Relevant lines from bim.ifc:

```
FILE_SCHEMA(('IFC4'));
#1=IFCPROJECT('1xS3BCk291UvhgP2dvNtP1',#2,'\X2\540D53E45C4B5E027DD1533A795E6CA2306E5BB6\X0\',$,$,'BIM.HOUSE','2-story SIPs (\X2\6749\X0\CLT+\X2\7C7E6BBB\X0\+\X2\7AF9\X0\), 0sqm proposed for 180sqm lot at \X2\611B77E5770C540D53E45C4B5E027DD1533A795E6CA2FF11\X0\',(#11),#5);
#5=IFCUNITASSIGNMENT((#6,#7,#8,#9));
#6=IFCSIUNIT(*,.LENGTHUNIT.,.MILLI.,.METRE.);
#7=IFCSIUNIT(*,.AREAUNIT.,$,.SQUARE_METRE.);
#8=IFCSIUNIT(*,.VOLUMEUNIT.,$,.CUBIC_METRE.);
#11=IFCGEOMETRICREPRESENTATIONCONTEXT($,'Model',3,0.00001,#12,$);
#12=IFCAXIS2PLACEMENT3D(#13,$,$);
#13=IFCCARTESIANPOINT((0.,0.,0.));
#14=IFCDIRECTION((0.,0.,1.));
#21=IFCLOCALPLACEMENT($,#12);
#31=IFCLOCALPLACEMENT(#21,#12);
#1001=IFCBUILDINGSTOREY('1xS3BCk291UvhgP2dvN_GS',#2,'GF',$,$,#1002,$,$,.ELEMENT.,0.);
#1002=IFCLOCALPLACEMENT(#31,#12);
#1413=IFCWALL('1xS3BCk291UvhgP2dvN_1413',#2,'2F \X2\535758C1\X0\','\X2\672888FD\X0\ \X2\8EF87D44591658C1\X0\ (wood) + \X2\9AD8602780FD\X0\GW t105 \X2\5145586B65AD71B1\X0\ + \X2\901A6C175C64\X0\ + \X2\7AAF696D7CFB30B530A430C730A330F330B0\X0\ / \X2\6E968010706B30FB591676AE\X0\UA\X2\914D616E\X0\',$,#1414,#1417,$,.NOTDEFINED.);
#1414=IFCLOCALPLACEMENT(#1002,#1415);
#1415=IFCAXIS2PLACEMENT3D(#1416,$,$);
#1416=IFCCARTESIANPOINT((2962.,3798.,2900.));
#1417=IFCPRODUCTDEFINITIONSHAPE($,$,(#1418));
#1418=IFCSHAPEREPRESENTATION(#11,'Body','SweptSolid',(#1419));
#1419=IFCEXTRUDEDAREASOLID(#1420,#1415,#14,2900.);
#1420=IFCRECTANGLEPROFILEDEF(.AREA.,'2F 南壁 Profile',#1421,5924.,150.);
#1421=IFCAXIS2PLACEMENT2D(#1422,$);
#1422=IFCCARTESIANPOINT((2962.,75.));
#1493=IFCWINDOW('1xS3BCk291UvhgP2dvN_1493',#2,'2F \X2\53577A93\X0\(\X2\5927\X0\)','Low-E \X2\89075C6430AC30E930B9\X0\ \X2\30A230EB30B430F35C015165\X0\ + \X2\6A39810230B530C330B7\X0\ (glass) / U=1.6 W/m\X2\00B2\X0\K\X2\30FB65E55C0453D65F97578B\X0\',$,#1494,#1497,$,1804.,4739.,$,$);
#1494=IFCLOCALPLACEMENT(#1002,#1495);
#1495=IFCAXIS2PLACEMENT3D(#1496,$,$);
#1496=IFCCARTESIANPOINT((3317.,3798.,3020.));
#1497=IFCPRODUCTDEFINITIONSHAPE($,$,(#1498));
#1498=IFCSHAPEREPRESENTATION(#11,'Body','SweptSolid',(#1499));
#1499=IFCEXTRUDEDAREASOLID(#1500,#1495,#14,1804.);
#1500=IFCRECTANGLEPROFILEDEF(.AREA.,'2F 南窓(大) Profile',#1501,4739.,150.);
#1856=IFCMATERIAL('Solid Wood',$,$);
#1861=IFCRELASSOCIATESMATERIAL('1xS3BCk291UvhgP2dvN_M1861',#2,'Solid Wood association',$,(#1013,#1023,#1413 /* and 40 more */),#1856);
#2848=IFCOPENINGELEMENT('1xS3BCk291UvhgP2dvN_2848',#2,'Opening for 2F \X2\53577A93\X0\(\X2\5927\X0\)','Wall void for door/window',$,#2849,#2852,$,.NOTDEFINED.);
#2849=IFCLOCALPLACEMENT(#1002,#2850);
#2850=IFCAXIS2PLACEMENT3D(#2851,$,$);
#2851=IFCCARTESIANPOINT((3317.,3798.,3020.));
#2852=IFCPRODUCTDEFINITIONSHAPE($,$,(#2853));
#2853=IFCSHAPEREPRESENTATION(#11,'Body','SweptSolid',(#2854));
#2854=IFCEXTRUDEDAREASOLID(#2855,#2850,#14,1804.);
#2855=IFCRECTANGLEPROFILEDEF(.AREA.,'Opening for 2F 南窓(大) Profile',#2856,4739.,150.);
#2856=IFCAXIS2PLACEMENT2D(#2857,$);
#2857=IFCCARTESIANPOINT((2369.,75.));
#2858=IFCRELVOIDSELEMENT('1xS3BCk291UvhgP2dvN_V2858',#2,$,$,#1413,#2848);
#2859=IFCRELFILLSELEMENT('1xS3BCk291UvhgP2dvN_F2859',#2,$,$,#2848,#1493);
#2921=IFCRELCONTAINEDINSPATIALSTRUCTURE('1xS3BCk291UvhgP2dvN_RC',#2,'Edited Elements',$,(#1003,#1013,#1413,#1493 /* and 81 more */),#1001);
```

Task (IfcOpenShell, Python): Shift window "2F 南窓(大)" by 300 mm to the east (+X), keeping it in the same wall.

```python
import ifcopenshell
import ifcopenshell.api.geometry
import ifcopenshell.util.placement
import ifcopenshell.util.unit

model = ifcopenshell.open("bim.ifc")
unit_scale = ifcopenshell.util.unit.calculate_unit_scale(model)

window = model.by_guid("1xS3BCk291UvhgP2dvN_1493")
opening = window.FillsVoids[0].RelatingOpeningElement
wall = opening.VoidsElements[0].RelatingBuildingElement

wall_matrix = ifcopenshell.util.placement.get_local_placement(wall.ObjectPlacement)
shift = wall_matrix[:3, 0] * 0.3 / unit_scale
before = ifcopenshell.util.placement.get_local_placement(window.ObjectPlacement)[:3, 3].copy()

# The window is not placed relative to its opening, so move both.
for product in (opening, window):
    matrix = ifcopenshell.util.placement.get_local_placement(product.ObjectPlacement)
    matrix[:3, 3] += shift
    ifcopenshell.api.geometry.edit_object_placement(model, product=product, matrix=matrix, is_si=False)

after = ifcopenshell.util.placement.get_local_placement(window.ObjectPlacement)[:3, 3]
print("window moved by", (after - before).round(3) + 0.0)

model.write("bim_updated.ifc")
```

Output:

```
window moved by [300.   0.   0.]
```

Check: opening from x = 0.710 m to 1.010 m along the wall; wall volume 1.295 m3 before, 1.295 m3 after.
